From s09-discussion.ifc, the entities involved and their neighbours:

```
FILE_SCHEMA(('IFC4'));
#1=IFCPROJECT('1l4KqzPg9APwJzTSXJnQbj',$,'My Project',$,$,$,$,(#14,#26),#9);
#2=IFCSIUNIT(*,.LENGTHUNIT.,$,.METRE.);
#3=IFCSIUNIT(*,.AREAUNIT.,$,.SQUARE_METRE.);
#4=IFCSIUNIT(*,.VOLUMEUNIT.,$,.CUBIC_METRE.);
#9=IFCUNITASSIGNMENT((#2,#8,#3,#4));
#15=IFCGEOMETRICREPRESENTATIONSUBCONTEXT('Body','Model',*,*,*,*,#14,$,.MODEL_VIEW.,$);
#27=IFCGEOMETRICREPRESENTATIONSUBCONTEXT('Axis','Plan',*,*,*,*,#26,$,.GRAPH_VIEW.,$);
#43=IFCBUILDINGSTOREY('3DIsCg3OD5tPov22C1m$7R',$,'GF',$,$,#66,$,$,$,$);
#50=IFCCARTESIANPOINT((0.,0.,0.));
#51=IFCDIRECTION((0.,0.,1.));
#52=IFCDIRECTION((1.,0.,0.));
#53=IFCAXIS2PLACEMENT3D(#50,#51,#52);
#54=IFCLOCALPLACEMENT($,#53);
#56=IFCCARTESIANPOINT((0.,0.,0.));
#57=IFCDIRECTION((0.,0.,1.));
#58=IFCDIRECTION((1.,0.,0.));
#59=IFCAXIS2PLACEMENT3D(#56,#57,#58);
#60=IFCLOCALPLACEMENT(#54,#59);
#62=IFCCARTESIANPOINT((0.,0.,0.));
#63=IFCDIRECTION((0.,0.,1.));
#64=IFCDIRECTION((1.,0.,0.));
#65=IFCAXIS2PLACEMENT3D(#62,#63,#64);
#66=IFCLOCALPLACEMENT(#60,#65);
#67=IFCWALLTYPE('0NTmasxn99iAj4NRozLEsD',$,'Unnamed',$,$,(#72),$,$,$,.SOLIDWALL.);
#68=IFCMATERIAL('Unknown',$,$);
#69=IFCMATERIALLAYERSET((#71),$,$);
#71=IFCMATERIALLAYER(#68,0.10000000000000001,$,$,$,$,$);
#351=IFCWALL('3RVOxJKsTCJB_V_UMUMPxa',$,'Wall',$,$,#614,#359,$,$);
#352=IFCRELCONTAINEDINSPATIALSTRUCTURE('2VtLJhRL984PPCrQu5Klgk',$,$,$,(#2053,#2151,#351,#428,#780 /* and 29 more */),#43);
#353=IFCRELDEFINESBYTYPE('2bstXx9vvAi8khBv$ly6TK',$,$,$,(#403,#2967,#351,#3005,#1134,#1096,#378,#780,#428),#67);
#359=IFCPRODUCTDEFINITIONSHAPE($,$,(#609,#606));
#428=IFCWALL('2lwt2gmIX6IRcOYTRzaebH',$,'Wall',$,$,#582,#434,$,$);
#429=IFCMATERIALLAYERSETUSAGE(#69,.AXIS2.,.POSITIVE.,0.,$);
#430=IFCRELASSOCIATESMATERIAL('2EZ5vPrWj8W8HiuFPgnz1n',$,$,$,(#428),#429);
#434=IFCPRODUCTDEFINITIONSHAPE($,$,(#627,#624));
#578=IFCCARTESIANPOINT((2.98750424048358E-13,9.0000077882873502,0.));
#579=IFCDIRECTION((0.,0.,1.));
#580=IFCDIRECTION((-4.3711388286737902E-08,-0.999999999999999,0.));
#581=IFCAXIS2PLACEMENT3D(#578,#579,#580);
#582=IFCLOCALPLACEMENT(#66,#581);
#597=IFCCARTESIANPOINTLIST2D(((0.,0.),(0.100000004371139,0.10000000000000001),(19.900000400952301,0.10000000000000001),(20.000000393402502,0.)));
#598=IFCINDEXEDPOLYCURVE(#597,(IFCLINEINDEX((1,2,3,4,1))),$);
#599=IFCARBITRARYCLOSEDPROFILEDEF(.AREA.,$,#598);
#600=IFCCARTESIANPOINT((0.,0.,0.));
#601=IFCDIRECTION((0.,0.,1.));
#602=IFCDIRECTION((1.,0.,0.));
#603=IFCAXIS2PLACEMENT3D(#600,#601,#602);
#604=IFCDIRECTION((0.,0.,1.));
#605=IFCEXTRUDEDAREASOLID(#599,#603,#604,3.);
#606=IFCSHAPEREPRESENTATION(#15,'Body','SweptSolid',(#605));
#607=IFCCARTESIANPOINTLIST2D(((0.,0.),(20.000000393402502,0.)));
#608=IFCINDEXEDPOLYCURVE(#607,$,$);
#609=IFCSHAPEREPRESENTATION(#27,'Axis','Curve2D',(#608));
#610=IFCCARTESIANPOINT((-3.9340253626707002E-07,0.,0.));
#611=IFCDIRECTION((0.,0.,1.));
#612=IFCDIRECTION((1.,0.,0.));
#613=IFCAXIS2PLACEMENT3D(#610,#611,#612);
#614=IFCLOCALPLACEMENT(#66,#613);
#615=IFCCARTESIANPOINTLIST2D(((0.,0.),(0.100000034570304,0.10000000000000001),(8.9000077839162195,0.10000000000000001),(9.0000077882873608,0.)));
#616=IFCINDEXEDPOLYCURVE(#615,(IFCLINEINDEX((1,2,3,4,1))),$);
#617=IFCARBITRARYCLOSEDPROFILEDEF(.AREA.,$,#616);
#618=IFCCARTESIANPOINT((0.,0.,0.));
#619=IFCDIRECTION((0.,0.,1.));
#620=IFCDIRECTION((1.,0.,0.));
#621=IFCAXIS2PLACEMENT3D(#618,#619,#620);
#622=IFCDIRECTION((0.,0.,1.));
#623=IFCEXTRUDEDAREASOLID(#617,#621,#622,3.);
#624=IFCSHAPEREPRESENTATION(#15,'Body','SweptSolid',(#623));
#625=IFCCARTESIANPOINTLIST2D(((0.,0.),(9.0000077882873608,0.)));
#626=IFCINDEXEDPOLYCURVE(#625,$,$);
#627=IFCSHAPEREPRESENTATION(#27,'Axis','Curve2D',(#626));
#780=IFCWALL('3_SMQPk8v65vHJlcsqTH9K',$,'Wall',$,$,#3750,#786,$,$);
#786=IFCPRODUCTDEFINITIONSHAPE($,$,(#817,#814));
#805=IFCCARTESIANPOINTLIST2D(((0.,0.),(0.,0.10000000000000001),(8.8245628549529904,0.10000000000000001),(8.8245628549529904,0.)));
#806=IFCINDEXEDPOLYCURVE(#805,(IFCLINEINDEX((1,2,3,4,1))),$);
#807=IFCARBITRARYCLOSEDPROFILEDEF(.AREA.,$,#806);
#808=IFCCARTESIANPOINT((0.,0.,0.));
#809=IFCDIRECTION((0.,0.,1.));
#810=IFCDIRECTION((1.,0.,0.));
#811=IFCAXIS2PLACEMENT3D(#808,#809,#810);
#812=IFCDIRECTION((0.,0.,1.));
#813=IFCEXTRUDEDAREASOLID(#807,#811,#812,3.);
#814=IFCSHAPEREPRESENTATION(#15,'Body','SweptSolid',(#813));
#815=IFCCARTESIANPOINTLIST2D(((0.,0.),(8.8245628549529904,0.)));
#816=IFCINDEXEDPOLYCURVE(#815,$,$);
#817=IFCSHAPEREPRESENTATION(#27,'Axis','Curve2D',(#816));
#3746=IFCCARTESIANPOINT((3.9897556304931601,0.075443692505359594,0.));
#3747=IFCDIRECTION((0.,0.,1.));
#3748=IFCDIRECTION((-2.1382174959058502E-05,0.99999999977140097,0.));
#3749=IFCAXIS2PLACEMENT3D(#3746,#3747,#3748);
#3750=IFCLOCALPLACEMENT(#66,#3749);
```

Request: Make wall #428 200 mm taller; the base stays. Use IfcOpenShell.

```python
import ifcopenshell
import ifcopenshell.geom
import ifcopenshell.util.representation
import ifcopenshell.util.shape
import ifcopenshell.util.unit

model = ifcopenshell.open("s09-discussion.ifc")
unit_scale = ifcopenshell.util.unit.calculate_unit_scale(model)
settings = ifcopenshell.geom.settings()


def volume(element):
    """Net volume in cubic metres, openings subtracted."""
    shape = ifcopenshell.geom.create_shape(settings, element)
    return ifcopenshell.util.shape.get_volume(shape.geometry)


wall = model.by_id(428)
before = volume(wall)

body = ifcopenshell.util.representation.get_representation(wall, "Model", "Body")
solid = body.Items[0]
old_height = solid.Depth
solid.Depth += 0.2 / unit_scale
after = volume(wall)

print(f"height {old_height:g} -> {solid.Depth:g}, volume {before:.3f} -> {after:.3f} m3")

model.write("s09-discussion_rev.ifc")
```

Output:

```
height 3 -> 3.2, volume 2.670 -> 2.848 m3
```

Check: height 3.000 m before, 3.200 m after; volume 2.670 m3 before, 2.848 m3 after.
